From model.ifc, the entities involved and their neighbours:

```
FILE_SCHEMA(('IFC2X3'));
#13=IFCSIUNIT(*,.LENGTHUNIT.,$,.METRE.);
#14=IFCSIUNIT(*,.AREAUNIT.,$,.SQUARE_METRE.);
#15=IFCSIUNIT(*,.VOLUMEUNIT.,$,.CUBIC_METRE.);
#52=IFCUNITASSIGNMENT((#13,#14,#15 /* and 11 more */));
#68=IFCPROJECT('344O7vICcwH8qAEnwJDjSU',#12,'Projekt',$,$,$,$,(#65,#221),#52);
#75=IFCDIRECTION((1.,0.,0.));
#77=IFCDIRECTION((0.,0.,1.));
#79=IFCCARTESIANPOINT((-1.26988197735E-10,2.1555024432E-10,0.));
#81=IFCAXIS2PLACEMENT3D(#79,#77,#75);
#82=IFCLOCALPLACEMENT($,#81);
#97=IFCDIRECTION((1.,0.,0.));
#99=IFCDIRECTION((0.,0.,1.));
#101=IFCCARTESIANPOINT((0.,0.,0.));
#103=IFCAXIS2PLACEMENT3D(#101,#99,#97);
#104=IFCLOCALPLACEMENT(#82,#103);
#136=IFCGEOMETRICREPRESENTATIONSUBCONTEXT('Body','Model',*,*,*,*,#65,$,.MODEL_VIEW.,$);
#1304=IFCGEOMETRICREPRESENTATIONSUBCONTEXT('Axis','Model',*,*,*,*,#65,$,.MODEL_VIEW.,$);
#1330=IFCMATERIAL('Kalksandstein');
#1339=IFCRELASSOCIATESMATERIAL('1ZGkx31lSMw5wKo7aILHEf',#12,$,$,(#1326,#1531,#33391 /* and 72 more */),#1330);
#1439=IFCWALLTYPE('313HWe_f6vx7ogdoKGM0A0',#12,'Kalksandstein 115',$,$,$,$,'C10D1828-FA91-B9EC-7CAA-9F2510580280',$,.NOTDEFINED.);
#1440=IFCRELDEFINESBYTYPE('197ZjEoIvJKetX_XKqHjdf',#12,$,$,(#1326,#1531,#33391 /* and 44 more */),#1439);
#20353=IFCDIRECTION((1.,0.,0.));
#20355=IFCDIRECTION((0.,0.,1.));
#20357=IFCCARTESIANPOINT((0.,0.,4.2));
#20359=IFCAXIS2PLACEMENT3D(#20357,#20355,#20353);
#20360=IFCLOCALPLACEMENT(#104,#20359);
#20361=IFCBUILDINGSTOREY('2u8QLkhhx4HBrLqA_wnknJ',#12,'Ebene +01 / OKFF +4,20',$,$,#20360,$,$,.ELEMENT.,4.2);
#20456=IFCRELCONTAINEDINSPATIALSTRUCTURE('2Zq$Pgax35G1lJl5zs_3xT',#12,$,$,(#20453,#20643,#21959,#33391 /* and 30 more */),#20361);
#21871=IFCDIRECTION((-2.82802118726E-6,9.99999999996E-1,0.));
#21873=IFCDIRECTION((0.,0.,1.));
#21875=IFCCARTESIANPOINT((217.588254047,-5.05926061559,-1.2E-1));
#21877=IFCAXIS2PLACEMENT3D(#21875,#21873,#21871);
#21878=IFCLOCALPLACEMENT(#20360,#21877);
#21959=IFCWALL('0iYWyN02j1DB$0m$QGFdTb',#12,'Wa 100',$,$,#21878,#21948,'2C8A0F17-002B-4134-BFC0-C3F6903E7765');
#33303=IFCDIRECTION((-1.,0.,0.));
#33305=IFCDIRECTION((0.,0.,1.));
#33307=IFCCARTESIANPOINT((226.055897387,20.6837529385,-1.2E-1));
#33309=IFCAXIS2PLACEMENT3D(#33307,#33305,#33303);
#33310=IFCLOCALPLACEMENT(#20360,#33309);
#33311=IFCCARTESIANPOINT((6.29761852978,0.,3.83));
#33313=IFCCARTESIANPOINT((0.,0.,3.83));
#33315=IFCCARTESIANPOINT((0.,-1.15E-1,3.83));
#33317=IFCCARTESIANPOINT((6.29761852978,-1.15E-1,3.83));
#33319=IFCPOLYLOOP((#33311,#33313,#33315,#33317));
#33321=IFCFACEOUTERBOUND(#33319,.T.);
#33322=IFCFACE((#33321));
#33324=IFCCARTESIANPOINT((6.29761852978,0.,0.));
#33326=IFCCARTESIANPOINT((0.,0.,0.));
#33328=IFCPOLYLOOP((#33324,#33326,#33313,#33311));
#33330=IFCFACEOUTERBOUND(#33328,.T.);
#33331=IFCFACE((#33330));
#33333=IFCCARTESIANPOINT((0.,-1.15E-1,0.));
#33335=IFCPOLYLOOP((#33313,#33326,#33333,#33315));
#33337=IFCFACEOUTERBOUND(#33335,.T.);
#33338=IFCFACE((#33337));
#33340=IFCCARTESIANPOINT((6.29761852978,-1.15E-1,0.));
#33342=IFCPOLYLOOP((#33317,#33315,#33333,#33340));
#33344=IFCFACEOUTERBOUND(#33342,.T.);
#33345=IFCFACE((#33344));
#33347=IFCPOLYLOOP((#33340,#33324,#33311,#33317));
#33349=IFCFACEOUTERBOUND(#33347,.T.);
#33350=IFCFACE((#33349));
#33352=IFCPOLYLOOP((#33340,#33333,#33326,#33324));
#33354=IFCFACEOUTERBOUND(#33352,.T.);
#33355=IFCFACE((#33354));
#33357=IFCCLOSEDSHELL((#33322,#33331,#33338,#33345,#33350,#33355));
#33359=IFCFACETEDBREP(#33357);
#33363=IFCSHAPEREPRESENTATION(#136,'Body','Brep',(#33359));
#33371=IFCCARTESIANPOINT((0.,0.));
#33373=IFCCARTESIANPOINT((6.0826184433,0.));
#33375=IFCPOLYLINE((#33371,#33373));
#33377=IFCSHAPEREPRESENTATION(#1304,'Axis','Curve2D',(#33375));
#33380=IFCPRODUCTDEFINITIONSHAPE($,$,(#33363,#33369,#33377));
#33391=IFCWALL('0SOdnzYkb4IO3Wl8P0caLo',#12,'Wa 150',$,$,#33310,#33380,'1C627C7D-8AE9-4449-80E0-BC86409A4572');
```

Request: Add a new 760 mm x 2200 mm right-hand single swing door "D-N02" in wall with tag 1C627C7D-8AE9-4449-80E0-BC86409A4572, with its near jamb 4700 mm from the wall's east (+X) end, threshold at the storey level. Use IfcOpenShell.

```python
import numpy as np
import ifcopenshell
import ifcopenshell.api.feature
import ifcopenshell.api.geometry
import ifcopenshell.api.root
import ifcopenshell.api.spatial
import ifcopenshell.api.type
import ifcopenshell.geom
import ifcopenshell.util.element
import ifcopenshell.util.placement
import ifcopenshell.util.representation
import ifcopenshell.util.shape
import ifcopenshell.util.unit

model = ifcopenshell.open("model.ifc")
unit_scale = ifcopenshell.util.unit.calculate_unit_scale(model)
settings = ifcopenshell.geom.settings()


def volume(element):
    """Net volume in cubic metres, openings subtracted."""
    shape = ifcopenshell.geom.create_shape(settings, element)
    return ifcopenshell.util.shape.get_volume(shape.geometry)


wall = model.by_guid("0SOdnzYkb4IO3Wl8P0caLo")
storey = ifcopenshell.util.element.get_container(wall, ifc_class="IfcBuildingStorey")
context = ifcopenshell.util.representation.get_context(model, "Model", "Body", "MODEL_VIEW")
before = volume(wall)

width, height, from_end, sill = 0.76, 2.2, 4.7, 0.0  # metres

# The wall runs along its own X axis, and the end named is its -X end.
wall_shape = ifcopenshell.geom.create_shape(settings, wall)
x, y, z = ifcopenshell.util.shape.get_vertices(wall_shape.geometry).T
start = x.min() + from_end
face, thickness = float(y.min()), float(y.max() - y.min())
wall_matrix = ifcopenshell.util.placement.get_local_placement(wall.ObjectPlacement)
level = ifcopenshell.util.placement.get_local_placement(storey.ObjectPlacement)[2, 3]


def in_wall(x, y):
    """Placement at x, y metres in the wall's axes, at sill height."""
    matrix = wall_matrix.copy()
    matrix[:, 3] = wall_matrix @ np.array([x / unit_scale, y / unit_scale, 0.0, 1.0])
    matrix[2, 3] = level + sill / unit_scale
    return matrix


# Opening: a box that overshoots both wall faces by 50 mm.
opening = ifcopenshell.api.root.create_entity(model, ifc_class="IfcOpeningElement")
box = ifcopenshell.api.geometry.add_wall_representation(
    model, context=context, length=width, height=height, thickness=thickness + 0.1
)
ifcopenshell.api.geometry.assign_representation(model, product=opening, representation=box)
ifcopenshell.api.geometry.edit_object_placement(model, product=opening, matrix=in_wall(start, face - 0.05), is_si=False)
ifcopenshell.api.feature.add_feature(model, feature=opening, element=wall)

door = ifcopenshell.api.root.create_entity(model, ifc_class="IfcDoor", name="D-N02")
door.OverallWidth, door.OverallHeight = width / unit_scale, height / unit_scale
body = ifcopenshell.api.geometry.add_door_representation(
    model,
    context=context,
    overall_width=door.OverallWidth,
    overall_height=door.OverallHeight,
    operation_type="SINGLE_SWING_RIGHT",
    lining_properties={"LiningDepth": thickness / unit_scale, "ThresholdDepth": thickness / unit_scale},
)
ifcopenshell.api.geometry.assign_representation(model, product=door, representation=body)
ifcopenshell.api.spatial.assign_container(model, products=[door], relating_structure=storey)
fills = ifcopenshell.api.feature.add_filling(model, opening=opening, element=door)
fills.OwnerHistory = door.OwnerHistory  # required in IFC2X3

# IFC2X3 keeps the operation on the door style.
style = ifcopenshell.api.root.create_entity(model, ifc_class="IfcDoorStyle", name="D-N02")
style.OperationType, style.ConstructionType = "SINGLE_SWING_RIGHT", "NOTDEFINED"
style.ParameterTakesPrecedence = style.Sizeable = False
ifcopenshell.api.type.assign_type(model, related_objects=[door], relating_type=style)

# The lining spans the wall, so the door starts at the wall face.
ifcopenshell.api.geometry.edit_object_placement(model, product=door, matrix=in_wall(start, face), is_si=False)

after = volume(wall)

print(f"wall volume {before:.3f} -> {after:.3f} m3")

model.write("model_updated.ifc")
```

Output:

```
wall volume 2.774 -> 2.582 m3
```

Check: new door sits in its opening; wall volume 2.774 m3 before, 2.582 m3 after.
